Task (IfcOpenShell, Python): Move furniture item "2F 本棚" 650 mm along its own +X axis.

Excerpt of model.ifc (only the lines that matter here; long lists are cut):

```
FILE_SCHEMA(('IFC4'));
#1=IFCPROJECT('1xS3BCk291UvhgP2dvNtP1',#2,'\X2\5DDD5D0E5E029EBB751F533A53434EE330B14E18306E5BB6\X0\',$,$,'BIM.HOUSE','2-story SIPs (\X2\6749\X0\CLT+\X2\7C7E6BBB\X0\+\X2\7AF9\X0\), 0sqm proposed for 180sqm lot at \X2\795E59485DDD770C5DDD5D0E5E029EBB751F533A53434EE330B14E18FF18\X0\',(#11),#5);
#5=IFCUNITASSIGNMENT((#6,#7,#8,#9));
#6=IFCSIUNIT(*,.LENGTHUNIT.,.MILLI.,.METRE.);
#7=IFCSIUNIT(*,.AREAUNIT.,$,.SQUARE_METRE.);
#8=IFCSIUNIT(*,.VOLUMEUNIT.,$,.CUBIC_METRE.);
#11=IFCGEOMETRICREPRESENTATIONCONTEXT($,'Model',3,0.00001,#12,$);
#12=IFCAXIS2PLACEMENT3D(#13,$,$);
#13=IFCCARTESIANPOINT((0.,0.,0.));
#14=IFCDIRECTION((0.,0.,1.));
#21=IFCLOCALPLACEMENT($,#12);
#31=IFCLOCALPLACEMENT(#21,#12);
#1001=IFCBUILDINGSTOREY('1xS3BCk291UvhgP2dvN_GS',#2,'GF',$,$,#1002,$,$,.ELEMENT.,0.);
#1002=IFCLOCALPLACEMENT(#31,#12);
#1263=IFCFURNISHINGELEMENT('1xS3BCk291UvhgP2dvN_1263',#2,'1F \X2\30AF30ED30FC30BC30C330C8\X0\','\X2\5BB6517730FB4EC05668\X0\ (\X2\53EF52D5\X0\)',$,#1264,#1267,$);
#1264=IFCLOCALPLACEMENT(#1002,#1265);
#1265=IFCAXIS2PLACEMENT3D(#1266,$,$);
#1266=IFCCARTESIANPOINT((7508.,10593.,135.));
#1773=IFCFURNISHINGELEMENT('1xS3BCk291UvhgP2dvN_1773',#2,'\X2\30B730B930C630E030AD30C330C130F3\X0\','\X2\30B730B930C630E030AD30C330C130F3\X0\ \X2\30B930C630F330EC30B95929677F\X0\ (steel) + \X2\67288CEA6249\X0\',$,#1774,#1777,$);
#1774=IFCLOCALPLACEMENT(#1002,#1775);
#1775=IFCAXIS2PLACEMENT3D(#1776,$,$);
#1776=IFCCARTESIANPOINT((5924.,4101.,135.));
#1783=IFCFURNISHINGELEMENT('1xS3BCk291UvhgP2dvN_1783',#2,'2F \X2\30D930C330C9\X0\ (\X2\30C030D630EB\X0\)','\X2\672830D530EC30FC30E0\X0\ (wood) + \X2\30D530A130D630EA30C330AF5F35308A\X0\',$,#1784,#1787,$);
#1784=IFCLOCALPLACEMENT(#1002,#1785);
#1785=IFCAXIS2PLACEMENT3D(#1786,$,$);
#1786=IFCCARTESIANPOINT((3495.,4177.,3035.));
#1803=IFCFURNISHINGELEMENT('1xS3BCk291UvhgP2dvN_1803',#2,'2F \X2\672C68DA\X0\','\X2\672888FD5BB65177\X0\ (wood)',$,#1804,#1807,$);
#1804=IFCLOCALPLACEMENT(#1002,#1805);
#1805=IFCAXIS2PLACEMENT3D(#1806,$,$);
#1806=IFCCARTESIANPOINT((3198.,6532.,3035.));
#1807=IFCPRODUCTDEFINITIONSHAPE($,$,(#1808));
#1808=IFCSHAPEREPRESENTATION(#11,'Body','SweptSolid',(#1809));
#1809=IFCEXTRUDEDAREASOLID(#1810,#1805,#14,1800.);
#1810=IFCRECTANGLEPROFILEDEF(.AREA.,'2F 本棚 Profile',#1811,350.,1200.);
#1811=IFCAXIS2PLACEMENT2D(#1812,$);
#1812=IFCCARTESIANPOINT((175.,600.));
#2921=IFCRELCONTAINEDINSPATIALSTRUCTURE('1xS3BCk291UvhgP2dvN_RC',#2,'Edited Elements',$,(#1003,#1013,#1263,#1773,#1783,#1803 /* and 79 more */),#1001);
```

```python
import ifcopenshell
import ifcopenshell.api.geometry
import ifcopenshell.util.placement

model = ifcopenshell.open("model.ifc")

item = model.by_guid("1xS3BCk291UvhgP2dvN_1803")
matrix = ifcopenshell.util.placement.get_local_placement(item.ObjectPlacement)
matrix[:3, 3] += matrix[:3, 0] * 650.0
ifcopenshell.api.geometry.edit_object_placement(model, product=item, matrix=matrix, is_si=False)

print(ifcopenshell.util.placement.get_local_placement(item.ObjectPlacement).round(3) + 0.0)

model.write("model_edited.ifc")
```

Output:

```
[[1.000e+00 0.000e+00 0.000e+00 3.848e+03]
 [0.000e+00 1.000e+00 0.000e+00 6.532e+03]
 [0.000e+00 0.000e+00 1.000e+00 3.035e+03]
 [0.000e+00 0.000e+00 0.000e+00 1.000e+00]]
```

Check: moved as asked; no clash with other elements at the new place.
